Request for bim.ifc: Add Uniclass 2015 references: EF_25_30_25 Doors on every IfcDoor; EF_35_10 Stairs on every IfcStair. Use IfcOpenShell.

First a look at what the model holds.

```python
import ifcopenshell

model = ifcopenshell.open("bim.ifc")
print(model.schema)
print("classifications:", [c.Name for c in model.by_type("IfcClassification")])
for ifc_class in ("IfcDoor", "IfcRoof", "IfcStair", "IfcWall", "IfcWindow"):
    print(ifc_class, len(model.by_type(ifc_class)))
```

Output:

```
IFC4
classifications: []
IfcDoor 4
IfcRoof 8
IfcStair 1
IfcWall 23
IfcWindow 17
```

```python
import ifcopenshell
import ifcopenshell.api.classification

model = ifcopenshell.open("bim.ifc")

system = ifcopenshell.api.classification.add_classification(model, classification="Uniclass 2015")

codes = {
    "IfcDoor": ("EF_25_30_25", "Doors"),
    "IfcStair": ("EF_35_10", "Stairs"),
}
for ifc_class, (code, name) in codes.items():
    products = model.by_type(ifc_class)
    ifcopenshell.api.classification.add_reference(
        model, products=products, classification=system, identification=code, name=name
    )
    print(code, len(products))

model.write("bim_v2.ifc")
```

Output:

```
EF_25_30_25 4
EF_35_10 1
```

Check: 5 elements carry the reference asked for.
